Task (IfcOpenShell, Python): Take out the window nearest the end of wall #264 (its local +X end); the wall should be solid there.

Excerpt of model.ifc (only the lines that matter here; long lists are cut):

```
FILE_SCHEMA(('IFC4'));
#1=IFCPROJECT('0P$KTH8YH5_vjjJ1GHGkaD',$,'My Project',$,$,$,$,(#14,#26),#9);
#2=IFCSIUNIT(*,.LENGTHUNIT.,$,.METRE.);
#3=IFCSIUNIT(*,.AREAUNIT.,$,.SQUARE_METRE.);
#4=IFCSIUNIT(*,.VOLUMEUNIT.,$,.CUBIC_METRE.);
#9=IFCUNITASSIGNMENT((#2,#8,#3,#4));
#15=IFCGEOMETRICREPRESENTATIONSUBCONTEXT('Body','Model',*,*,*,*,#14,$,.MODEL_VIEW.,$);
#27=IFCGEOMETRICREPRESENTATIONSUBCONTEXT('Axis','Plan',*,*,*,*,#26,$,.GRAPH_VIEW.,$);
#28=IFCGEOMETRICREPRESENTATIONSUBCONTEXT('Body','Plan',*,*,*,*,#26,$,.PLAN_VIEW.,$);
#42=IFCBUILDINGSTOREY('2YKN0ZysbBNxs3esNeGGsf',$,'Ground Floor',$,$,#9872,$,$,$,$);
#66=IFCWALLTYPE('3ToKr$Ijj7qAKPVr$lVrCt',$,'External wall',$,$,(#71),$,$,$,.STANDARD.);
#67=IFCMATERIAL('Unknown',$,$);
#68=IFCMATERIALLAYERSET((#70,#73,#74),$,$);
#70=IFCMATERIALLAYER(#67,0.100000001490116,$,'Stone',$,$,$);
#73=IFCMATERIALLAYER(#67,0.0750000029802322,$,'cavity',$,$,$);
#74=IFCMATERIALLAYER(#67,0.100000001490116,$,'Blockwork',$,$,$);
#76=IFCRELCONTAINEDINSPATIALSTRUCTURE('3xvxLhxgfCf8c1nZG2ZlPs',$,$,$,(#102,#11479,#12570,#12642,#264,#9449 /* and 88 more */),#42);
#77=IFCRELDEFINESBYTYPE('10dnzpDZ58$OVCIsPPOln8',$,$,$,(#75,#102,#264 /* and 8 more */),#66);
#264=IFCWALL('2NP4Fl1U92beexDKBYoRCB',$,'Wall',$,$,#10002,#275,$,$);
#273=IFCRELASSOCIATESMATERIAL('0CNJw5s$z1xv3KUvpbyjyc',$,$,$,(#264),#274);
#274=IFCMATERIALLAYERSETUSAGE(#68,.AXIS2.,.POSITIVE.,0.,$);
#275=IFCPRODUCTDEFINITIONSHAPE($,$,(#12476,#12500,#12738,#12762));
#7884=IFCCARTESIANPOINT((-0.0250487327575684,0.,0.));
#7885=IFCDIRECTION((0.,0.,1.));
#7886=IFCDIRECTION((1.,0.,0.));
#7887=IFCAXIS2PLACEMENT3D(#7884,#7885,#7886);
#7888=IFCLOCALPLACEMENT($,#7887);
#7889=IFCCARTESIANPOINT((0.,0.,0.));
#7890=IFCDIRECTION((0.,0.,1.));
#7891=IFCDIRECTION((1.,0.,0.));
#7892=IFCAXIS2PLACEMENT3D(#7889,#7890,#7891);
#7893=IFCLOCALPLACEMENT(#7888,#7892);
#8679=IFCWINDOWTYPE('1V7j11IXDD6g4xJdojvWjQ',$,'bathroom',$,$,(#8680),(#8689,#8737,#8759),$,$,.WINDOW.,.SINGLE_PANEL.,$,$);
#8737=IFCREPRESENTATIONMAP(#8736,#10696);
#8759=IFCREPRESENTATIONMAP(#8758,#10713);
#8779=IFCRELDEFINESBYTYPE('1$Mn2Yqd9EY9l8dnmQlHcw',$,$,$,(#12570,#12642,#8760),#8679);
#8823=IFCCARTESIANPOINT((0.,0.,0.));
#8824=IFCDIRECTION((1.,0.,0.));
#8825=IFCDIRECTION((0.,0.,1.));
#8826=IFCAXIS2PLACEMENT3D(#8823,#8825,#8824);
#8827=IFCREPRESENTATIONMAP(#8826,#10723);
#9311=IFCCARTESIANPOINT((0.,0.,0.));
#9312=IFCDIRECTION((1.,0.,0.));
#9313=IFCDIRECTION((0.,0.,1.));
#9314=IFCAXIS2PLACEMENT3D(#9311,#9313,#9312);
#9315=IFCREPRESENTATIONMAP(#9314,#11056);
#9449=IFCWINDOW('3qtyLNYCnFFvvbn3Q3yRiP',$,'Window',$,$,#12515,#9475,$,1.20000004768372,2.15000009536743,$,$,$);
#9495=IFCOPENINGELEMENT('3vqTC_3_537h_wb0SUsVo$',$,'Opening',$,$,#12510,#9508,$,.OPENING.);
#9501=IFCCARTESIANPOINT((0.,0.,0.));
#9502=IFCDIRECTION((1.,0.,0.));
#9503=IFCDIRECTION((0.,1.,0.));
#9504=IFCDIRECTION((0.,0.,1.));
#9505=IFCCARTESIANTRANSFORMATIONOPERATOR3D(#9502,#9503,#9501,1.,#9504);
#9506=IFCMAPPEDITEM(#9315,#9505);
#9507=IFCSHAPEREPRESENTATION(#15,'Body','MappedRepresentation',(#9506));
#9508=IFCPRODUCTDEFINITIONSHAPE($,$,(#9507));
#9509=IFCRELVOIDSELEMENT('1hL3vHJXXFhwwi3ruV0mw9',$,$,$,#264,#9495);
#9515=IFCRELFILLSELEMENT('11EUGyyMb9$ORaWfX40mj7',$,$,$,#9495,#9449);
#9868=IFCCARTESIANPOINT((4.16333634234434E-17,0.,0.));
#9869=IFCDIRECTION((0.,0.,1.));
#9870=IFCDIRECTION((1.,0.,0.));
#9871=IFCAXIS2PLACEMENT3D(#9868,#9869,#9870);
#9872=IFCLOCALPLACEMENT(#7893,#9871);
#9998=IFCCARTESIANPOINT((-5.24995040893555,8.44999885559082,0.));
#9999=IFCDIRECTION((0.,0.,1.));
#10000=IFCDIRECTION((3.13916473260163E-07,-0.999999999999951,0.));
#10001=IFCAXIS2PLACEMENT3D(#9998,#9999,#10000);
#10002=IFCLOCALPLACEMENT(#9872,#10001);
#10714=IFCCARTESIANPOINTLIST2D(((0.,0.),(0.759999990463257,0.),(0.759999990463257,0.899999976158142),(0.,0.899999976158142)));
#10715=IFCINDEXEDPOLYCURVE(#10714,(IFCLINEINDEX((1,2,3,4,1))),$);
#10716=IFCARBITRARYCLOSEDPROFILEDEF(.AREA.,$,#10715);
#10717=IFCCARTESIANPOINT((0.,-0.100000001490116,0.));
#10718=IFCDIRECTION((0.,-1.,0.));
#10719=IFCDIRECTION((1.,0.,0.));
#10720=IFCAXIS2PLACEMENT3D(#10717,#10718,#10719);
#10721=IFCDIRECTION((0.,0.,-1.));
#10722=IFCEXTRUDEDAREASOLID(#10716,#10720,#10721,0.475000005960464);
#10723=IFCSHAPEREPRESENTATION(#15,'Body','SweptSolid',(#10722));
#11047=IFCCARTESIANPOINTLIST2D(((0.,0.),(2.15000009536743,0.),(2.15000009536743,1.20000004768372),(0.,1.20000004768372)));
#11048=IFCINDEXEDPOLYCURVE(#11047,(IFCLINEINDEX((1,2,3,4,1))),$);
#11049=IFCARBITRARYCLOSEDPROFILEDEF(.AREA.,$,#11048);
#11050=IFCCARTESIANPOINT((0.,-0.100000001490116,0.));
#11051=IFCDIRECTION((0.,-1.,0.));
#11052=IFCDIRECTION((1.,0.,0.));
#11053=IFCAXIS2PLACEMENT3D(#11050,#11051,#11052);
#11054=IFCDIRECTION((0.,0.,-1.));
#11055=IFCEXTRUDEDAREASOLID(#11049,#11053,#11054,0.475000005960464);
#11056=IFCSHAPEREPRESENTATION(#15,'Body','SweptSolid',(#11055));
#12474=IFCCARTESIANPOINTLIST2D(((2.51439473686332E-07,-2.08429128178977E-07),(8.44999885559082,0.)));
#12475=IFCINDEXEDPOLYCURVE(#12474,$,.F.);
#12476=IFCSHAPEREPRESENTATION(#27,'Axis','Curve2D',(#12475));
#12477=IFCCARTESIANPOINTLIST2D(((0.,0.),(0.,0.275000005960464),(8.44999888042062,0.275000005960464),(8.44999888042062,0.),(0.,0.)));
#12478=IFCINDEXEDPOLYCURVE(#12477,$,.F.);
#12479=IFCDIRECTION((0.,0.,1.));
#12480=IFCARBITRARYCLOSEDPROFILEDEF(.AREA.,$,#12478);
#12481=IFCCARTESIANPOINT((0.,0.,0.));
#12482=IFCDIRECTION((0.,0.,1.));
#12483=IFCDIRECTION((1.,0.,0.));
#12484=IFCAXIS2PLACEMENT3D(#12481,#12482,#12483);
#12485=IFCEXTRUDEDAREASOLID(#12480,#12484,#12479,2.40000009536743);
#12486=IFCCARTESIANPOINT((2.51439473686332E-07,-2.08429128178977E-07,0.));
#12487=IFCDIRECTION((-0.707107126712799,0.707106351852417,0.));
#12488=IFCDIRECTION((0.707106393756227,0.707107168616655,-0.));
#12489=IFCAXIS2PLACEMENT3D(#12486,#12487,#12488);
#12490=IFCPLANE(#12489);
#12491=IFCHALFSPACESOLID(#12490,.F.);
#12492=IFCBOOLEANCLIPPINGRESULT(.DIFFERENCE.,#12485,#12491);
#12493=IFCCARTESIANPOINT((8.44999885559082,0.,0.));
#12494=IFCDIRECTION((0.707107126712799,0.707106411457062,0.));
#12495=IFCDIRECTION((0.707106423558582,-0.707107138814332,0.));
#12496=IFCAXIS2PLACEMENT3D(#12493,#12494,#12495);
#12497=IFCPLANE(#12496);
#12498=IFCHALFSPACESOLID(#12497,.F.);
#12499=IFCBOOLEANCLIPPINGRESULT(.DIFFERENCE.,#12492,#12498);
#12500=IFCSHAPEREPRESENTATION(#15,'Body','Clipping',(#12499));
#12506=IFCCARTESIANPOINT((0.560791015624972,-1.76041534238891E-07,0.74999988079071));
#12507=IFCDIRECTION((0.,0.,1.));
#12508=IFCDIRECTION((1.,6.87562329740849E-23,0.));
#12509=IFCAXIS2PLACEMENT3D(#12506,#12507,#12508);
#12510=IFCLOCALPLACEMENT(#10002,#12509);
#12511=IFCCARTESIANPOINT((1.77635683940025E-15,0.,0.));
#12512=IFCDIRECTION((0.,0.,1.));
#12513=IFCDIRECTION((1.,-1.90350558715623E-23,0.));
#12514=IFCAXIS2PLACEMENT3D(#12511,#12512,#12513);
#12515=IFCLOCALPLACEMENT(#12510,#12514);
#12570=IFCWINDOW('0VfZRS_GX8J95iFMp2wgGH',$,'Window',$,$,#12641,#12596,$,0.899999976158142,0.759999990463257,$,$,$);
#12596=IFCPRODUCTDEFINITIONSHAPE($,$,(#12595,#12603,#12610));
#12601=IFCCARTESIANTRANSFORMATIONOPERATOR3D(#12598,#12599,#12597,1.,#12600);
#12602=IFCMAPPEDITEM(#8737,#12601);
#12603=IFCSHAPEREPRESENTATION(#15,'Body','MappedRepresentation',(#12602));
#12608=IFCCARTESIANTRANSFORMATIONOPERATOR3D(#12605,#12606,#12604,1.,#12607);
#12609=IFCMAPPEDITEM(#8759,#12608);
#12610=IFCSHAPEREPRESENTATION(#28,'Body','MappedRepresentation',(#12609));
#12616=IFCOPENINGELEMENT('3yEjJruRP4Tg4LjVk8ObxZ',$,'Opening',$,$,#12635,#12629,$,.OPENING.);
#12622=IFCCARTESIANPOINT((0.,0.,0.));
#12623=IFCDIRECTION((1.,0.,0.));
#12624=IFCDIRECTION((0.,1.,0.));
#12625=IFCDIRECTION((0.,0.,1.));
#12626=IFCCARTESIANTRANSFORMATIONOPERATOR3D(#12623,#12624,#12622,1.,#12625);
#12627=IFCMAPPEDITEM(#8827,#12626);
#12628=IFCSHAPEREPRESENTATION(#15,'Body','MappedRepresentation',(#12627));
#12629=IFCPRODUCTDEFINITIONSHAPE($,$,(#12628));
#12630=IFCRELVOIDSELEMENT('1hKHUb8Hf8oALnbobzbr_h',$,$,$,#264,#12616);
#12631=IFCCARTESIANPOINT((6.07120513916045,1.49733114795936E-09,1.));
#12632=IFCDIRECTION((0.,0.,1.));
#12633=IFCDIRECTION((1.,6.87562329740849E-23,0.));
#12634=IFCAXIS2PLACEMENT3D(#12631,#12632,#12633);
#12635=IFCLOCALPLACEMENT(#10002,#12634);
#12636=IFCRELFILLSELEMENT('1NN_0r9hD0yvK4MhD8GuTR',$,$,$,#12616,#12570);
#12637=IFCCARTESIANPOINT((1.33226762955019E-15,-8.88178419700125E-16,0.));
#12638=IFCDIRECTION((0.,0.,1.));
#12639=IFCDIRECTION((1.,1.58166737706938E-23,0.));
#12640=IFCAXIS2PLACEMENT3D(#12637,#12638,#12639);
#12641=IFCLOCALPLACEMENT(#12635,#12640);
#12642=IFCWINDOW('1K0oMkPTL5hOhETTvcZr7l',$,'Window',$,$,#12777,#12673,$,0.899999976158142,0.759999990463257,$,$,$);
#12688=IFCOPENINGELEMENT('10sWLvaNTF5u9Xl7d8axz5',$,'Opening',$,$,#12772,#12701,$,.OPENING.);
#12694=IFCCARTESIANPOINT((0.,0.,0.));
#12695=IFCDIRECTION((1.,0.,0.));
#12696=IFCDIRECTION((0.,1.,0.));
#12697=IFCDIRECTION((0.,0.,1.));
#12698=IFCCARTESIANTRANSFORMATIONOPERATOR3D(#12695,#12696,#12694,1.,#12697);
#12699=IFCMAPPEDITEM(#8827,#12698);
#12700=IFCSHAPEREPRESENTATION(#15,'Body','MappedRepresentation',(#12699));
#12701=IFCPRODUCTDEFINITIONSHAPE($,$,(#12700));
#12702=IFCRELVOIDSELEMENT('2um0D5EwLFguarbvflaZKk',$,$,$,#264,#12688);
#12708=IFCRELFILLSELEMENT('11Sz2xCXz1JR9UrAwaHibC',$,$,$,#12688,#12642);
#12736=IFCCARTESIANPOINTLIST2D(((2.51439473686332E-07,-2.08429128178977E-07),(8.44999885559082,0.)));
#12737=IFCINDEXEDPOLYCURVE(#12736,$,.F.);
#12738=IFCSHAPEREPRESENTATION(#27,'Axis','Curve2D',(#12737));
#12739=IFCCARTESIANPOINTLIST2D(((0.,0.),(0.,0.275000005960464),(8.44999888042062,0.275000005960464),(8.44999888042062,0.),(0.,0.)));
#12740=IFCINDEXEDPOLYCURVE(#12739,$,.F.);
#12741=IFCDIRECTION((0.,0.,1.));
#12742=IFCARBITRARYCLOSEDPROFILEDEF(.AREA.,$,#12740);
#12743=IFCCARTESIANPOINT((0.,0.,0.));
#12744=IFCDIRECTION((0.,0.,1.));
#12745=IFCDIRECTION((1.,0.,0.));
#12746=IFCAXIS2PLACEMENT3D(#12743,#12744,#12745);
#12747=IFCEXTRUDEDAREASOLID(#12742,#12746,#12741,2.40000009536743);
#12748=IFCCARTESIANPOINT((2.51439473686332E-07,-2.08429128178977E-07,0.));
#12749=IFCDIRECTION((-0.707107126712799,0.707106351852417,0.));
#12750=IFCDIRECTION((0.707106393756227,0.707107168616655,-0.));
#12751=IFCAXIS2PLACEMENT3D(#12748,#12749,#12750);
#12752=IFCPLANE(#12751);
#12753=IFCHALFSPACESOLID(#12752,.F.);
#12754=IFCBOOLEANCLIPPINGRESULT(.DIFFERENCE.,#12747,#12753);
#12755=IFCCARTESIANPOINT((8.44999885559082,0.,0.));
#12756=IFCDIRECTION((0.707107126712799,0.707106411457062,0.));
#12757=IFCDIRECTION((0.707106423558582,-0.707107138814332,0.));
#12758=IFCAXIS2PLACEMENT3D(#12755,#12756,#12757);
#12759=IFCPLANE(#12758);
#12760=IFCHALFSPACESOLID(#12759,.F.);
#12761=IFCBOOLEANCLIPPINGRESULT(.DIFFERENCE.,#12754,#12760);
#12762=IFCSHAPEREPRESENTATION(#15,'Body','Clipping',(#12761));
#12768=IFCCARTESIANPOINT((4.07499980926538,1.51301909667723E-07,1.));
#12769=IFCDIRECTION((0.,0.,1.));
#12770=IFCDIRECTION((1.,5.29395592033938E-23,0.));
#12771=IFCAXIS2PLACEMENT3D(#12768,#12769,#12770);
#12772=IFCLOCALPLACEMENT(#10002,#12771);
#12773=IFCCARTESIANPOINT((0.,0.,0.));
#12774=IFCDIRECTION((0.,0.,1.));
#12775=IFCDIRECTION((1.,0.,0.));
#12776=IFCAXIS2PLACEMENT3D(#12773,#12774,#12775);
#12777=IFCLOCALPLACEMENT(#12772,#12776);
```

```python
import ifcopenshell
import ifcopenshell.api.feature
import ifcopenshell.api.root
import ifcopenshell.geom
import ifcopenshell.util.shape

model = ifcopenshell.open("model.ifc")
settings = ifcopenshell.geom.settings()


def volume(element):
    """Net volume in cubic metres, openings subtracted."""
    shape = ifcopenshell.geom.create_shape(settings, element)
    return ifcopenshell.util.shape.get_volume(shape.geometry)


window = model.by_guid("0VfZRS_GX8J95iFMp2wgGH")
opening = window.FillsVoids[0].RelatingOpeningElement
wall = opening.VoidsElements[0].RelatingBuildingElement
before = volume(wall)

ifcopenshell.api.root.remove_product(model, product=window)
ifcopenshell.api.feature.remove_feature(model, feature=opening)

after = volume(wall)

print(f"wall volume {before:.3f} -> {after:.3f} m3")

model.write("model_updated.ifc")
```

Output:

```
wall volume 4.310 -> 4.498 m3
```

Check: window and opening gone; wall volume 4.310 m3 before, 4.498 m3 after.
